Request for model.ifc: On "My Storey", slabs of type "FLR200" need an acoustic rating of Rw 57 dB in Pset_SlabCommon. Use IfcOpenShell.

First a look at what the model holds.

```python
import ifcopenshell
import ifcopenshell.util.element

model = ifcopenshell.open("model.ifc")
print(model.schema)
storey = next(s for s in model.by_type("IfcBuildingStorey") if s.Name == "My Storey")
slabs = [e for e in ifcopenshell.util.element.get_decomposition(storey) if e.is_a("IfcSlab")]
seen = {}
for e in slabs:
    element_type = ifcopenshell.util.element.get_type(e)
    key = (element_type.Name if element_type != e and element_type else None, ifcopenshell.util.element.get_pset(e, "Pset_SlabCommon", "AcousticRating"))
    seen[key] = seen.get(key, 0) + 1
for (name, value), count in sorted(seen.items(), key=str):
    print(count, "x", name, "|", value)
```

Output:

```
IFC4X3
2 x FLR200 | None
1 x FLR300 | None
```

```python
import ifcopenshell
import ifcopenshell.api.pset
import ifcopenshell.util.element

model = ifcopenshell.open("model.ifc")

storey = next(s for s in model.by_type("IfcBuildingStorey") if s.Name == "My Storey")
slabs = [e for e in ifcopenshell.util.element.get_decomposition(storey) if e.is_a("IfcSlab")]

count = 0
for e in slabs:
    element_type = ifcopenshell.util.element.get_type(e)
    if element_type in (None, e) or element_type.Name != "FLR200":
        continue
    # add_pset returns the element's existing set when there is one.
    pset = ifcopenshell.api.pset.add_pset(model, product=e, name="Pset_SlabCommon")
    ifcopenshell.api.pset.edit_pset(model, pset=pset, properties={"AcousticRating": "Rw 57 dB"})
    count += 1

print(count, "slabs updated")

model.write("model_edited.ifc")
```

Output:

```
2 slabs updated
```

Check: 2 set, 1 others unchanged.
